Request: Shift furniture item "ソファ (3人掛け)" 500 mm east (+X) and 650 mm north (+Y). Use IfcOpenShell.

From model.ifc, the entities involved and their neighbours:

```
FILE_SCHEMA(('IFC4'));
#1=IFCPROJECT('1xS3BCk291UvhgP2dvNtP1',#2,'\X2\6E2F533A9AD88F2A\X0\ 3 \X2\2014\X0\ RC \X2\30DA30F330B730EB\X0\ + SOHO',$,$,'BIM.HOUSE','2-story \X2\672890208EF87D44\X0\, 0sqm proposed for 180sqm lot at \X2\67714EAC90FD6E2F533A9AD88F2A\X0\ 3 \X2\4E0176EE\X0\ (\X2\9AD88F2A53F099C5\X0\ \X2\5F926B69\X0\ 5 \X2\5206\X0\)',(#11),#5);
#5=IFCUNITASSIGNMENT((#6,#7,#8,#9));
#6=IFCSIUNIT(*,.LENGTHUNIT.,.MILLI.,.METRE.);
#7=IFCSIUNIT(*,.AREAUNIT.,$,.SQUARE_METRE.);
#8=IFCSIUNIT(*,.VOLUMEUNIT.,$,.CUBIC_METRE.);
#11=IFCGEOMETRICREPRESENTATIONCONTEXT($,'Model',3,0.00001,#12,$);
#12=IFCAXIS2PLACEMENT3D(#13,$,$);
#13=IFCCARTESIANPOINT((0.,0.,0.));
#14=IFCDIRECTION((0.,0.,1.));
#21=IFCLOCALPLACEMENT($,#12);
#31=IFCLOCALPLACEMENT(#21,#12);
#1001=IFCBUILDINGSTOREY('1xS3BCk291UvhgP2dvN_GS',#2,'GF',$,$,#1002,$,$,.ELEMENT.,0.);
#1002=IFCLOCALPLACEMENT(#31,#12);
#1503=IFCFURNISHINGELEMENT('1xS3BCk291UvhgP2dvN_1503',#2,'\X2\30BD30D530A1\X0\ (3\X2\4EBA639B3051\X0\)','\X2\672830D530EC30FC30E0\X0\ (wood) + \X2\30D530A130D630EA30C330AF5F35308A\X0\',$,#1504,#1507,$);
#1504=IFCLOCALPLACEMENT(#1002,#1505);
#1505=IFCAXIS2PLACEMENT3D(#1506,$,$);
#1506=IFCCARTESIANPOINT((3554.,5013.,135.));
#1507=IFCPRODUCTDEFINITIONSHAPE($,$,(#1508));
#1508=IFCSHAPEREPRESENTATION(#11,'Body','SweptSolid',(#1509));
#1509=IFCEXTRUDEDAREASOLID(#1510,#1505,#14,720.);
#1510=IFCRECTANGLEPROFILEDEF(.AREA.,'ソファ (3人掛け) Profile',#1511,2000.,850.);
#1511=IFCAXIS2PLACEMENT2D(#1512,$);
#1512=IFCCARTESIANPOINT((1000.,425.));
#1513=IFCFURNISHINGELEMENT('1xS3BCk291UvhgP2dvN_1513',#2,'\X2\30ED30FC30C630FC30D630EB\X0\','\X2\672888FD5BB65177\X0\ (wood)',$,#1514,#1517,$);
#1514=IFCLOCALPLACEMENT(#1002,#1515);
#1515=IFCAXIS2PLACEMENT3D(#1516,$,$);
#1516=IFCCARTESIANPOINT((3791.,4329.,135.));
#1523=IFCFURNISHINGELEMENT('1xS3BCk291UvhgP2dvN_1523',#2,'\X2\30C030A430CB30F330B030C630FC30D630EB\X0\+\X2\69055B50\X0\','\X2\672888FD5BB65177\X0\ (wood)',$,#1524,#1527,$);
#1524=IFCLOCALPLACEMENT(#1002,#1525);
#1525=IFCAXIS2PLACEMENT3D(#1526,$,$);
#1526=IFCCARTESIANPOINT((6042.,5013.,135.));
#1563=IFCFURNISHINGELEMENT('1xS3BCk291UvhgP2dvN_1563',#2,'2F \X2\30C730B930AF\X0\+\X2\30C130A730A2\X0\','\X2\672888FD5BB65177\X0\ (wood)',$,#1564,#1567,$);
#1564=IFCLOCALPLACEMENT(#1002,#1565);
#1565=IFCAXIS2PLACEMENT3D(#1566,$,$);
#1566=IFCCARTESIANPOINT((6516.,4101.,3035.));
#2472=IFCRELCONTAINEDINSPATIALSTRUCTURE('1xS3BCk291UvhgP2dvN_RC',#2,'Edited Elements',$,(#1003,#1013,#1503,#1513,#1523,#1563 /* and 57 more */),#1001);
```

```python
import ifcopenshell
import ifcopenshell.api.geometry
import ifcopenshell.util.placement
import ifcopenshell.util.unit

model = ifcopenshell.open("model.ifc")
unit_scale = ifcopenshell.util.unit.calculate_unit_scale(model)

item = model.by_guid("1xS3BCk291UvhgP2dvN_1503")
matrix = ifcopenshell.util.placement.get_local_placement(item.ObjectPlacement)
matrix[0, 3] += 0.5 / unit_scale
matrix[1, 3] += 0.65 / unit_scale
ifcopenshell.api.geometry.edit_object_placement(model, product=item, matrix=matrix, is_si=False)

print(ifcopenshell.util.placement.get_local_placement(item.ObjectPlacement).round(3) + 0.0)

model.write("model_rev.ifc")
```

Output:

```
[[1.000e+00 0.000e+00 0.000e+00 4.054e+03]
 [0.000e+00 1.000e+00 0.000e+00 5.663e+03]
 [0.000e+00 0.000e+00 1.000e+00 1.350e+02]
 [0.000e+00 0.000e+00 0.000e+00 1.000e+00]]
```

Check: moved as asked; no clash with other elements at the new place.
